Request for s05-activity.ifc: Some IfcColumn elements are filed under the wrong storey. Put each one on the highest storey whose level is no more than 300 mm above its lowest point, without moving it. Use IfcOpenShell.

First a look at what the model holds.

```python
import ifcopenshell
import ifcopenshell.util.element
import ifcopenshell.util.placement

model = ifcopenshell.open("s05-activity.ifc")
print(model.schema)
for storey in model.by_type("IfcBuildingStorey"):
    level = ifcopenshell.util.placement.get_storey_elevation(storey)
    count = sum(e.is_a("IfcColumn") for e in ifcopenshell.util.element.get_contained(storey))
    print(storey.id(), storey.Name, round(level, 3), count, sep=" | ")
```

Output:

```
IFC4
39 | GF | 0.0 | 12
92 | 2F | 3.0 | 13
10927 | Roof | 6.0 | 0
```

```python
import ifcopenshell
import ifcopenshell.api.spatial
import ifcopenshell.geom
import ifcopenshell.util.element
import ifcopenshell.util.placement
import ifcopenshell.util.shape
import ifcopenshell.util.unit

model = ifcopenshell.open("s05-activity.ifc")
unit_scale = ifcopenshell.util.unit.calculate_unit_scale(model)
settings = ifcopenshell.geom.settings()

levels = sorted(
    ((ifcopenshell.util.placement.get_storey_elevation(s) * unit_scale, s) for s in model.by_type("IfcBuildingStorey")),
    key=lambda pair: pair[0],
)

for e in model.by_type("IfcColumn"):
    current = e.ContainedInStructure[0].RelatingStructure if e.ContainedInStructure else None
    if current is None or not current.is_a("IfcBuildingStorey"):
        continue
    shape = ifcopenshell.geom.create_shape(settings, e)
    bottom = ifcopenshell.util.shape.get_shape_bottom_elevation(shape, shape.geometry)
    below = [s for level, s in levels if level <= bottom + 0.3]
    storey = below[-1] if below else levels[0][1]
    if storey != current:
        # assign_container keeps the world position.
        ifcopenshell.api.spatial.assign_container(model, products=[e], relating_structure=storey)
        print(e.id(), current.Name, "->", storey.Name)

model.write("s05-activity_rev.ifc")
```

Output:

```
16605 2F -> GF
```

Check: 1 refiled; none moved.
